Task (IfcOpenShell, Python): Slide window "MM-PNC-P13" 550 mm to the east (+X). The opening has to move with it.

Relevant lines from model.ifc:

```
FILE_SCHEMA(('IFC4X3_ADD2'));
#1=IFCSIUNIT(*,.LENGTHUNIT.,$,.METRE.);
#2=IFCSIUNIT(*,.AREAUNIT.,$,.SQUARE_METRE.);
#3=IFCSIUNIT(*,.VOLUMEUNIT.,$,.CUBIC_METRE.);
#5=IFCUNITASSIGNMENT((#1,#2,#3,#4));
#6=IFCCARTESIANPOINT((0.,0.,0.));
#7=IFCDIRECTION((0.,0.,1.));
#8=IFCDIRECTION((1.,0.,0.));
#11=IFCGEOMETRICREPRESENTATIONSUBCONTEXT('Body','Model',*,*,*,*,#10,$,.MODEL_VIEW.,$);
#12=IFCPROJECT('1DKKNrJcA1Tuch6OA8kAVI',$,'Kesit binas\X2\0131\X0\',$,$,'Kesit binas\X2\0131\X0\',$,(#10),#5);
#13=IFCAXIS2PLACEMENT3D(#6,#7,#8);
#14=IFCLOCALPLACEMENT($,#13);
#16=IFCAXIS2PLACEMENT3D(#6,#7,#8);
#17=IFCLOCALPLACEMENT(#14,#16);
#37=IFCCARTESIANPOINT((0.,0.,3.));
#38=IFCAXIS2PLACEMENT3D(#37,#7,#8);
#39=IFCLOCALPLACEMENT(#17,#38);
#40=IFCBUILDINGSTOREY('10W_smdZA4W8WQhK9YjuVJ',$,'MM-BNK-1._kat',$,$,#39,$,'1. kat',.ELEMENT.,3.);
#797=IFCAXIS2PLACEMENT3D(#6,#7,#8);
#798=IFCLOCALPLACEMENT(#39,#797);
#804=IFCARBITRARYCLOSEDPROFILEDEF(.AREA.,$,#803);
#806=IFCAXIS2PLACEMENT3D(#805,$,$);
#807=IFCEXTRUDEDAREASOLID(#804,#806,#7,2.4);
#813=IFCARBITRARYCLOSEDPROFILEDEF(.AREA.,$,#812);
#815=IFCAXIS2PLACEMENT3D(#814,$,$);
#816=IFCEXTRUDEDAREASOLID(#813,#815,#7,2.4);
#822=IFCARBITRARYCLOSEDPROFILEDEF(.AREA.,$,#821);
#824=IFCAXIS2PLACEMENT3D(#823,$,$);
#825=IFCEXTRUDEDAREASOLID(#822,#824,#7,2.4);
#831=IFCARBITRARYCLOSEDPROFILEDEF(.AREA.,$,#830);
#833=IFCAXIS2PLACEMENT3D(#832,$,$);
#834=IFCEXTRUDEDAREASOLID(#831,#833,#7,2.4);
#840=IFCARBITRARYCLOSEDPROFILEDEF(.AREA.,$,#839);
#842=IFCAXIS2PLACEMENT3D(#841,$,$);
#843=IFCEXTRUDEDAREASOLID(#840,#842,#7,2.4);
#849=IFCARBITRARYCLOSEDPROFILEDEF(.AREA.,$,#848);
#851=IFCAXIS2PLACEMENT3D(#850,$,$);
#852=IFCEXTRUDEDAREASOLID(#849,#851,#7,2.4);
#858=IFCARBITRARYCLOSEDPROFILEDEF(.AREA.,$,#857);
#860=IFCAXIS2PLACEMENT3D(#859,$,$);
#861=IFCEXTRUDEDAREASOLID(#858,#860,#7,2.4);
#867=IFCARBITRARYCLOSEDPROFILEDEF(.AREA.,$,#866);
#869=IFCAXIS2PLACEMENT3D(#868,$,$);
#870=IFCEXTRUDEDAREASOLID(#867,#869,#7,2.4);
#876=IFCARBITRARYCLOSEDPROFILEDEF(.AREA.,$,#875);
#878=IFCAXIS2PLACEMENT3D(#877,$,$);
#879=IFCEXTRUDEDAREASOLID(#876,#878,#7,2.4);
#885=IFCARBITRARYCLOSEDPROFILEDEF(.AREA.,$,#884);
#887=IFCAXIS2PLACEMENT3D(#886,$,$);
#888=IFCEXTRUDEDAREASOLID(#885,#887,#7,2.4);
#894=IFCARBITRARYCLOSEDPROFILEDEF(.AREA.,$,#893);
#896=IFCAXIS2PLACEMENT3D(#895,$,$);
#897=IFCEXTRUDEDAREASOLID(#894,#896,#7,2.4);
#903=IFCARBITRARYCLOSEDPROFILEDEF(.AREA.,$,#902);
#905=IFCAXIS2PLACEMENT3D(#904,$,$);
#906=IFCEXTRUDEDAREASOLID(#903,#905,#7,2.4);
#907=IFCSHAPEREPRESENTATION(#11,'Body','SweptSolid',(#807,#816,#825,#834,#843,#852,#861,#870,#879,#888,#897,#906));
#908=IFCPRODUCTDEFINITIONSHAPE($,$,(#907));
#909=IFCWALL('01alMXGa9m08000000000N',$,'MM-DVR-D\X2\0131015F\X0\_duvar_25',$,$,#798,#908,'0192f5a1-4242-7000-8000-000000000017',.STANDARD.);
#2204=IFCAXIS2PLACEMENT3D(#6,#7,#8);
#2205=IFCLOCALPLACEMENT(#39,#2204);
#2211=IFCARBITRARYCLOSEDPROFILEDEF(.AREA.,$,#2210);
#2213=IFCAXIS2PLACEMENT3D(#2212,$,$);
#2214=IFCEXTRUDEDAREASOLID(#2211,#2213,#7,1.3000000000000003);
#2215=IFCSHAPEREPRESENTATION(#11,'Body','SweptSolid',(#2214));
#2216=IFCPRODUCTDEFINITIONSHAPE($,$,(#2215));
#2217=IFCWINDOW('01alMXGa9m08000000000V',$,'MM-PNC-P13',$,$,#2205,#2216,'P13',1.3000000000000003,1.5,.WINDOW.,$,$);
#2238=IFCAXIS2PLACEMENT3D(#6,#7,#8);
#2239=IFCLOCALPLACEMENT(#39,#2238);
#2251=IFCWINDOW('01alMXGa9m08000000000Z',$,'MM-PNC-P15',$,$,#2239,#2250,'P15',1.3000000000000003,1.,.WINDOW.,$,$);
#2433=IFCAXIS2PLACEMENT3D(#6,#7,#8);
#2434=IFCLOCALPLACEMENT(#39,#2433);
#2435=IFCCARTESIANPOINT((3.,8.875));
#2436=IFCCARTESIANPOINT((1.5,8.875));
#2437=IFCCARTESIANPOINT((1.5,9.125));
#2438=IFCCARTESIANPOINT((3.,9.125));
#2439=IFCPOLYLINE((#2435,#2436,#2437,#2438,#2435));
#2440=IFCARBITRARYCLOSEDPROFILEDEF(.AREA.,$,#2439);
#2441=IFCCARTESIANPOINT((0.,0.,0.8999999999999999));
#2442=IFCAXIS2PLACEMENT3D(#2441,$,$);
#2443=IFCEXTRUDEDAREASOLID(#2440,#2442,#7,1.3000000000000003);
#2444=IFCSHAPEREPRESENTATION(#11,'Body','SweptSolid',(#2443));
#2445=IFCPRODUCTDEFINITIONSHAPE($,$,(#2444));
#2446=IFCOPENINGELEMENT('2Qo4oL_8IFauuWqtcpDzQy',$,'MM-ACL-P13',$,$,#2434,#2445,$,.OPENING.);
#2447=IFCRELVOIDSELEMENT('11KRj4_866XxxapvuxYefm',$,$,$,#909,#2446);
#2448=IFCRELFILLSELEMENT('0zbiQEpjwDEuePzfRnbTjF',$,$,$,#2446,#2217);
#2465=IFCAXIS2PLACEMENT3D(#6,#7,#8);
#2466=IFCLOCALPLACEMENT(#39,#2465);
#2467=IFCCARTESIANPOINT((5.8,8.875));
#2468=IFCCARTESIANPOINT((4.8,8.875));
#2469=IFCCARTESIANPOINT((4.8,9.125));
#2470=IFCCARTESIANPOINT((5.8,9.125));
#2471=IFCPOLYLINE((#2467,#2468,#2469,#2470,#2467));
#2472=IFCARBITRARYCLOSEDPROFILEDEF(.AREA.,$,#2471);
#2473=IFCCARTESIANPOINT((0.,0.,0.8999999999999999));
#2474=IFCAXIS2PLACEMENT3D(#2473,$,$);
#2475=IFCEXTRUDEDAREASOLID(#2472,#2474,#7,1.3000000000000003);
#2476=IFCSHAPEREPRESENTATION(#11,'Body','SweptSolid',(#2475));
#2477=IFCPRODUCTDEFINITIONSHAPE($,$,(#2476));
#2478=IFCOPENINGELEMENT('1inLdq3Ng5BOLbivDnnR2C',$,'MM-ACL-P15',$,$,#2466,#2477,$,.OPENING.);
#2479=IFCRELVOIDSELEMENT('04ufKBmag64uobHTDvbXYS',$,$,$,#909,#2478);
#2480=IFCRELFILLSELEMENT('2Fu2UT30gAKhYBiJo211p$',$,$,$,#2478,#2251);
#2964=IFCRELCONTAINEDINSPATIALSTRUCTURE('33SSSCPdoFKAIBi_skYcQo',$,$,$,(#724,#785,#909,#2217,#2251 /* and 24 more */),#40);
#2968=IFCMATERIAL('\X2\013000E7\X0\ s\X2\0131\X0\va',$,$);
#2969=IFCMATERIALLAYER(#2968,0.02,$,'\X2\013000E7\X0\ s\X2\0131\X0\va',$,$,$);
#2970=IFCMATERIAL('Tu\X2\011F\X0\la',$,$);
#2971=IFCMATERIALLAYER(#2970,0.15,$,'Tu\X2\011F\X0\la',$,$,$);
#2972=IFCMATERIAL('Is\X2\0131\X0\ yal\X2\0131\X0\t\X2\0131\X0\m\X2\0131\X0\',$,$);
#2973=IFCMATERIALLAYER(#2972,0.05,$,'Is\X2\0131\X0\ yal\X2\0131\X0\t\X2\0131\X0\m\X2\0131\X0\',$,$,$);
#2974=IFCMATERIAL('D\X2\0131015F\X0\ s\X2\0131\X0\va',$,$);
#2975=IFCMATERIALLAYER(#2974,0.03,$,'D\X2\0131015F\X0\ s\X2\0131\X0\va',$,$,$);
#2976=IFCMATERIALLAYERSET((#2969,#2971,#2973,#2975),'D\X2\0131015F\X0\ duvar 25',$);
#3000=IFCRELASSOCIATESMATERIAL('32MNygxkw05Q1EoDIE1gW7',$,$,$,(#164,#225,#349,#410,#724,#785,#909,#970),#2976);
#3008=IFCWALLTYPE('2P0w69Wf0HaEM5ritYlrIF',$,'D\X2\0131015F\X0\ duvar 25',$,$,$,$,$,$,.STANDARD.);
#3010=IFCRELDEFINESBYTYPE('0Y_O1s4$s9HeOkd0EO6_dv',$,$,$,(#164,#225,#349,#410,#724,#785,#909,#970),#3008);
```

```python
import ifcopenshell
import ifcopenshell.api.geometry
import ifcopenshell.util.placement
import ifcopenshell.util.unit

model = ifcopenshell.open("model.ifc")
unit_scale = ifcopenshell.util.unit.calculate_unit_scale(model)

window = model.by_guid("01alMXGa9m08000000000V")
opening = window.FillsVoids[0].RelatingOpeningElement
wall = opening.VoidsElements[0].RelatingBuildingElement

wall_matrix = ifcopenshell.util.placement.get_local_placement(wall.ObjectPlacement)
shift = wall_matrix[:3, 0] * 0.55 / unit_scale
before = ifcopenshell.util.placement.get_local_placement(window.ObjectPlacement)[:3, 3].copy()

# The window is not placed relative to its opening, so move both.
for product in (opening, window):
    matrix = ifcopenshell.util.placement.get_local_placement(product.ObjectPlacement)
    matrix[:3, 3] += shift
    ifcopenshell.api.geometry.edit_object_placement(model, product=product, matrix=matrix, is_si=False)

after = ifcopenshell.util.placement.get_local_placement(window.ObjectPlacement)[:3, 3]
print("window moved by", (after - before).round(3) + 0.0)

model.write("model_edited.ifc")
```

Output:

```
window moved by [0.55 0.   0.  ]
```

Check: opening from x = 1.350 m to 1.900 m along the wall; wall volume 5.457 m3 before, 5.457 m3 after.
